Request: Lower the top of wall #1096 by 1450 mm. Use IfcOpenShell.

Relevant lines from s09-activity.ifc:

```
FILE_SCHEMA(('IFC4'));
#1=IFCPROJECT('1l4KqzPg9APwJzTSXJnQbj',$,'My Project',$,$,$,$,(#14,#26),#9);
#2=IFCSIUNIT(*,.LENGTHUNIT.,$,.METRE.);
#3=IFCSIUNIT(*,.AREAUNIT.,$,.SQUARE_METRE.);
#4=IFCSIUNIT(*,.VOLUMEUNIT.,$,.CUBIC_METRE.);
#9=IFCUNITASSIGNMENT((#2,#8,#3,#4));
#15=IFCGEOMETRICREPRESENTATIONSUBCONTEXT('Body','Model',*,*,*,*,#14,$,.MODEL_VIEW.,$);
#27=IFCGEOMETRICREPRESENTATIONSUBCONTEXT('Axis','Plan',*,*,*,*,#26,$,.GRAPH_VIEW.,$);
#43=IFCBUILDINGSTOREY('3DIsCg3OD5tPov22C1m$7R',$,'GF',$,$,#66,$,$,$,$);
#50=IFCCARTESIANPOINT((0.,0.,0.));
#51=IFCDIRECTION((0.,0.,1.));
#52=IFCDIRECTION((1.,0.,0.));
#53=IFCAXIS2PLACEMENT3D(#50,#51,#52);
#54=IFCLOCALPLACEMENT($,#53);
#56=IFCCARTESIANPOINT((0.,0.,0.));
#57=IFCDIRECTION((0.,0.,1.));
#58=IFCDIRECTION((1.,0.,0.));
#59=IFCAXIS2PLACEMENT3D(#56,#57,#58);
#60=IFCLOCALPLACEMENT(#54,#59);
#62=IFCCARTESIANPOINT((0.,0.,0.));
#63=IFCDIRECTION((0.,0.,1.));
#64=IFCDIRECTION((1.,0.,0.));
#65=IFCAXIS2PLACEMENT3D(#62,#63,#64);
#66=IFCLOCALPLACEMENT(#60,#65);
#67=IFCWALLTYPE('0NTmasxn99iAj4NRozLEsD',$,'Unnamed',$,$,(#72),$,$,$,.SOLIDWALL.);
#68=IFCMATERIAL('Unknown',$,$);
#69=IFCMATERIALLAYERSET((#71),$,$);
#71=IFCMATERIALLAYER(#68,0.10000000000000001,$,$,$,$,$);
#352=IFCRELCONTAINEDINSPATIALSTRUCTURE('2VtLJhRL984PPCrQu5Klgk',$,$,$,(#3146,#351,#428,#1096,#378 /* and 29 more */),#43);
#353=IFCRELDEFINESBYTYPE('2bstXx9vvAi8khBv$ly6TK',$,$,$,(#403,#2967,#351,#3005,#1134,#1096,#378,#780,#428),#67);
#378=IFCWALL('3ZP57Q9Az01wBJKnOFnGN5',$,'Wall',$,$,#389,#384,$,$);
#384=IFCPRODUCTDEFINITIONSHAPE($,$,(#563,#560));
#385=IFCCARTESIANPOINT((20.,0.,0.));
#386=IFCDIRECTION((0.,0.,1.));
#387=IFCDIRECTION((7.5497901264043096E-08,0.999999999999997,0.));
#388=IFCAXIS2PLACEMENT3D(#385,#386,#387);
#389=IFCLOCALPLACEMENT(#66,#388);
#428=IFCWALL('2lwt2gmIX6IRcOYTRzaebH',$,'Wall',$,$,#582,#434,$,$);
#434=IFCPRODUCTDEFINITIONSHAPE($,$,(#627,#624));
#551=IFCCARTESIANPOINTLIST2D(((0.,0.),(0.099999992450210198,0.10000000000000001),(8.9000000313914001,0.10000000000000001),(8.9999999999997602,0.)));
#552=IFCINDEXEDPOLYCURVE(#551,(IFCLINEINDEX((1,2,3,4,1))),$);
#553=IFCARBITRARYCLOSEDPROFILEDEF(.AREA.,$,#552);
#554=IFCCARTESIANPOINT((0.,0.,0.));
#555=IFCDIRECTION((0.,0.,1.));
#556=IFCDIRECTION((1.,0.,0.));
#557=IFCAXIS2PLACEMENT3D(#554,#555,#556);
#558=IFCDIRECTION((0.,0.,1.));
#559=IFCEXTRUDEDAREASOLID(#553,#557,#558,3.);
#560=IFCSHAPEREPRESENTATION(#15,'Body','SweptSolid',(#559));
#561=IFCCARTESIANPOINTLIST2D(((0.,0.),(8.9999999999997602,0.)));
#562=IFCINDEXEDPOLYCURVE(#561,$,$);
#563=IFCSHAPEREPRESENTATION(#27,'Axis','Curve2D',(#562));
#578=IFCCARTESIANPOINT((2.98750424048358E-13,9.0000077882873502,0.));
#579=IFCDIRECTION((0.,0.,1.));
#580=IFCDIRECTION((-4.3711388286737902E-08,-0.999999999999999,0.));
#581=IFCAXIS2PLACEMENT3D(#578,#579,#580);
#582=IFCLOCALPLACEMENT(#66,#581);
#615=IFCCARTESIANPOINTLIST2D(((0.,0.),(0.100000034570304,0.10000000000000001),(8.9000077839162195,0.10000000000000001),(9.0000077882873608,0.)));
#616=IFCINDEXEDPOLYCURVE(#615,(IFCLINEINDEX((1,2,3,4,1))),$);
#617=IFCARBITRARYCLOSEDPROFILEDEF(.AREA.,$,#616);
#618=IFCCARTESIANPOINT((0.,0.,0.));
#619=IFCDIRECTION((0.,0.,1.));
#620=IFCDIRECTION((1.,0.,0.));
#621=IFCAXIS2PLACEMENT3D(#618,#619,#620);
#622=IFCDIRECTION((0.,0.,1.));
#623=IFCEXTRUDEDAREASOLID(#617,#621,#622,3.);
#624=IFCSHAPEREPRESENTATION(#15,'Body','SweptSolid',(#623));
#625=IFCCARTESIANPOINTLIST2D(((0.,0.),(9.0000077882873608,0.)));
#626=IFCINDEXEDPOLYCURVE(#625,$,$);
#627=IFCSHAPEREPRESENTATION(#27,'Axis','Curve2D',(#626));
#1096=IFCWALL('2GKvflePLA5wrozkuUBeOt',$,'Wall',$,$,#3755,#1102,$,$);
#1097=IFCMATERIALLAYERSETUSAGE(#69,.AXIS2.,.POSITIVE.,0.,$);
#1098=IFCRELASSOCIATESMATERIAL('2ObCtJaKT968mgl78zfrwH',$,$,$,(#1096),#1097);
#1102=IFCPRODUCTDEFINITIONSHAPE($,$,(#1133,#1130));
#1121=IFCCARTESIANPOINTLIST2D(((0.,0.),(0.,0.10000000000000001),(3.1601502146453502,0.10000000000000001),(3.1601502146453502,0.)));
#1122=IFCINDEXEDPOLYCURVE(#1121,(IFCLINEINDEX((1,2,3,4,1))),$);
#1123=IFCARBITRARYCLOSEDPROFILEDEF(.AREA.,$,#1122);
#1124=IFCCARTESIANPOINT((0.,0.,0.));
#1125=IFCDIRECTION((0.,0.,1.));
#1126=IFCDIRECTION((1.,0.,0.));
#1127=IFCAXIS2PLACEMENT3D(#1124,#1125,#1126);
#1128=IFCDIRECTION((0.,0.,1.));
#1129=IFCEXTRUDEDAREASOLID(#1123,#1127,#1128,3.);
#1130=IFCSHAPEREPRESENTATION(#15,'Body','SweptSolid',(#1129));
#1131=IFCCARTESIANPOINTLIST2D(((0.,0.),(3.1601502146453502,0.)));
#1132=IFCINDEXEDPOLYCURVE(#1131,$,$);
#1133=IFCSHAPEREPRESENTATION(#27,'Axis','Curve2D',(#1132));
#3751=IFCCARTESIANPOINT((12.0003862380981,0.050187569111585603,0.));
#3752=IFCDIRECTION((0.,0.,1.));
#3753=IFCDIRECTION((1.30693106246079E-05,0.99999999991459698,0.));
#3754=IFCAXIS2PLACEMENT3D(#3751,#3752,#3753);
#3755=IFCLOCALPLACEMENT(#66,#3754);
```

```python
import ifcopenshell
import ifcopenshell.geom
import ifcopenshell.util.representation
import ifcopenshell.util.shape
import ifcopenshell.util.unit

model = ifcopenshell.open("s09-activity.ifc")
unit_scale = ifcopenshell.util.unit.calculate_unit_scale(model)
settings = ifcopenshell.geom.settings()


def volume(element):
    """Net volume in cubic metres, openings subtracted."""
    shape = ifcopenshell.geom.create_shape(settings, element)
    return ifcopenshell.util.shape.get_volume(shape.geometry)


wall = model.by_guid("2GKvflePLA5wrozkuUBeOt")
before = volume(wall)

body = ifcopenshell.util.representation.get_representation(wall, "Model", "Body")
solid = body.Items[0]
old_height = solid.Depth
solid.Depth -= 1.45 / unit_scale
after = volume(wall)

print(f"height {old_height:g} -> {solid.Depth:g}, volume {before:.3f} -> {after:.3f} m3")

model.write("s09-activity_rev.ifc")
```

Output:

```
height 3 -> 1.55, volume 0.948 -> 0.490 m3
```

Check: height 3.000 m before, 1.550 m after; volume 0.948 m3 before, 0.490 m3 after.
